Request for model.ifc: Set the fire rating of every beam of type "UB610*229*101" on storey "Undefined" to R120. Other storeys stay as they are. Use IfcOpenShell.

First a look at what the model holds.

```python
import ifcopenshell
import ifcopenshell.util.element

model = ifcopenshell.open("model.ifc")
print(model.schema)
storey = next(s for s in model.by_type("IfcBuildingStorey") if s.Name == "Undefined")
beams = [e for e in ifcopenshell.util.element.get_decomposition(storey) if e.is_a("IfcBeam")]
seen = {}
for e in beams:
    element_type = ifcopenshell.util.element.get_type(e)
    key = (element_type.Name if element_type != e and element_type else None, ifcopenshell.util.element.get_pset(e, "Pset_BeamCommon", "FireRating"))
    seen[key] = seen.get(key, 0) + 1
for (name, value), count in sorted(seen.items(), key=str):
    print(count, "x", name, "|", value)
```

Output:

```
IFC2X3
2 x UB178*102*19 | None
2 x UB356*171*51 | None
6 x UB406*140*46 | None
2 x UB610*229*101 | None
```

```python
import ifcopenshell
import ifcopenshell.api.pset
import ifcopenshell.util.element

model = ifcopenshell.open("model.ifc")

storey = next(s for s in model.by_type("IfcBuildingStorey") if s.Name == "Undefined")
beams = [e for e in ifcopenshell.util.element.get_decomposition(storey) if e.is_a("IfcBeam")]

count = 0
for e in beams:
    element_type = ifcopenshell.util.element.get_type(e)
    if element_type in (None, e) or element_type.Name != "UB610*229*101":
        continue
    # add_pset returns the element's existing set when there is one.
    pset = ifcopenshell.api.pset.add_pset(model, product=e, name="Pset_BeamCommon")
    ifcopenshell.api.pset.edit_pset(model, pset=pset, properties={"FireRating": "R120"})
    count += 1

print(count, "beams updated")

model.write("model-out.ifc")
```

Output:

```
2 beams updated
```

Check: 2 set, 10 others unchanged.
